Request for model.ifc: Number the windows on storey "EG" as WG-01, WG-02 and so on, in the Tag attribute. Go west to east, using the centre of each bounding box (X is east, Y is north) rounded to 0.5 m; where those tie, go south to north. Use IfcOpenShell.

First a look at what the model holds.

```python
import ifcopenshell
import ifcopenshell.util.element
import ifcopenshell.util.placement

model = ifcopenshell.open("model.ifc")
print(model.schema)
storey = next(s for s in model.by_type("IfcBuildingStorey") if s.Name == "EG")
windows = [e for e in ifcopenshell.util.element.get_decomposition(storey) if e.is_a("IfcWindow")]
for e in sorted(windows, key=lambda e: e.id()):
    origin = ifcopenshell.util.placement.get_local_placement(e.ObjectPlacement)[:3, 3]
    print(e.id(), e.Tag, e.Name, origin.round(2) + 0.0, sep=" | ")
```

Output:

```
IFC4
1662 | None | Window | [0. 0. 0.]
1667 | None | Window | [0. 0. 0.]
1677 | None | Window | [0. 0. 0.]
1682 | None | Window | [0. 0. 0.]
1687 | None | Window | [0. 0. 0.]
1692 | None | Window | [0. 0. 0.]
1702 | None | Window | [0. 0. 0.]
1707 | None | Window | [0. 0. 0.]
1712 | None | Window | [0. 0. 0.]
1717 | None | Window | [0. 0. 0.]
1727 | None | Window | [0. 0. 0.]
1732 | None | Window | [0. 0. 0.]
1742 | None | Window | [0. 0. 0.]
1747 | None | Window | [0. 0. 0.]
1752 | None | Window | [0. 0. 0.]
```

```python
import ifcopenshell
import ifcopenshell.geom
import ifcopenshell.util.element
import ifcopenshell.util.shape

model = ifcopenshell.open("model.ifc")
settings = ifcopenshell.geom.settings()
settings.set("use-world-coords", True)


def centre(element):
    shape = ifcopenshell.geom.create_shape(settings, element)
    return ifcopenshell.util.shape.get_bbox_centroid(shape.geometry)


storey = next(s for s in model.by_type("IfcBuildingStorey") if s.Name == "EG")
windows = [e for e in ifcopenshell.util.element.get_decomposition(storey) if e.is_a("IfcWindow")]

# Insertion points can sit at a corner or the storey origin, so sort by the geometry (in metres).
centres = {e: centre(e) for e in windows}
windows.sort(key=lambda e: (round(centres[e][0] / 0.5), centres[e][1]))

for i, e in enumerate(windows, start=1):
    number = f"WG-{i:02d}"
    e.Tag = number
    print(e.id(), number)

model.write("model_edited.ifc")
```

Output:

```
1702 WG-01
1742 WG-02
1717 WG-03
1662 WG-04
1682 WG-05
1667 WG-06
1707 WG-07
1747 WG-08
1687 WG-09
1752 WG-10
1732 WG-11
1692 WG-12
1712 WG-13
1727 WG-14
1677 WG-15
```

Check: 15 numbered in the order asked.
